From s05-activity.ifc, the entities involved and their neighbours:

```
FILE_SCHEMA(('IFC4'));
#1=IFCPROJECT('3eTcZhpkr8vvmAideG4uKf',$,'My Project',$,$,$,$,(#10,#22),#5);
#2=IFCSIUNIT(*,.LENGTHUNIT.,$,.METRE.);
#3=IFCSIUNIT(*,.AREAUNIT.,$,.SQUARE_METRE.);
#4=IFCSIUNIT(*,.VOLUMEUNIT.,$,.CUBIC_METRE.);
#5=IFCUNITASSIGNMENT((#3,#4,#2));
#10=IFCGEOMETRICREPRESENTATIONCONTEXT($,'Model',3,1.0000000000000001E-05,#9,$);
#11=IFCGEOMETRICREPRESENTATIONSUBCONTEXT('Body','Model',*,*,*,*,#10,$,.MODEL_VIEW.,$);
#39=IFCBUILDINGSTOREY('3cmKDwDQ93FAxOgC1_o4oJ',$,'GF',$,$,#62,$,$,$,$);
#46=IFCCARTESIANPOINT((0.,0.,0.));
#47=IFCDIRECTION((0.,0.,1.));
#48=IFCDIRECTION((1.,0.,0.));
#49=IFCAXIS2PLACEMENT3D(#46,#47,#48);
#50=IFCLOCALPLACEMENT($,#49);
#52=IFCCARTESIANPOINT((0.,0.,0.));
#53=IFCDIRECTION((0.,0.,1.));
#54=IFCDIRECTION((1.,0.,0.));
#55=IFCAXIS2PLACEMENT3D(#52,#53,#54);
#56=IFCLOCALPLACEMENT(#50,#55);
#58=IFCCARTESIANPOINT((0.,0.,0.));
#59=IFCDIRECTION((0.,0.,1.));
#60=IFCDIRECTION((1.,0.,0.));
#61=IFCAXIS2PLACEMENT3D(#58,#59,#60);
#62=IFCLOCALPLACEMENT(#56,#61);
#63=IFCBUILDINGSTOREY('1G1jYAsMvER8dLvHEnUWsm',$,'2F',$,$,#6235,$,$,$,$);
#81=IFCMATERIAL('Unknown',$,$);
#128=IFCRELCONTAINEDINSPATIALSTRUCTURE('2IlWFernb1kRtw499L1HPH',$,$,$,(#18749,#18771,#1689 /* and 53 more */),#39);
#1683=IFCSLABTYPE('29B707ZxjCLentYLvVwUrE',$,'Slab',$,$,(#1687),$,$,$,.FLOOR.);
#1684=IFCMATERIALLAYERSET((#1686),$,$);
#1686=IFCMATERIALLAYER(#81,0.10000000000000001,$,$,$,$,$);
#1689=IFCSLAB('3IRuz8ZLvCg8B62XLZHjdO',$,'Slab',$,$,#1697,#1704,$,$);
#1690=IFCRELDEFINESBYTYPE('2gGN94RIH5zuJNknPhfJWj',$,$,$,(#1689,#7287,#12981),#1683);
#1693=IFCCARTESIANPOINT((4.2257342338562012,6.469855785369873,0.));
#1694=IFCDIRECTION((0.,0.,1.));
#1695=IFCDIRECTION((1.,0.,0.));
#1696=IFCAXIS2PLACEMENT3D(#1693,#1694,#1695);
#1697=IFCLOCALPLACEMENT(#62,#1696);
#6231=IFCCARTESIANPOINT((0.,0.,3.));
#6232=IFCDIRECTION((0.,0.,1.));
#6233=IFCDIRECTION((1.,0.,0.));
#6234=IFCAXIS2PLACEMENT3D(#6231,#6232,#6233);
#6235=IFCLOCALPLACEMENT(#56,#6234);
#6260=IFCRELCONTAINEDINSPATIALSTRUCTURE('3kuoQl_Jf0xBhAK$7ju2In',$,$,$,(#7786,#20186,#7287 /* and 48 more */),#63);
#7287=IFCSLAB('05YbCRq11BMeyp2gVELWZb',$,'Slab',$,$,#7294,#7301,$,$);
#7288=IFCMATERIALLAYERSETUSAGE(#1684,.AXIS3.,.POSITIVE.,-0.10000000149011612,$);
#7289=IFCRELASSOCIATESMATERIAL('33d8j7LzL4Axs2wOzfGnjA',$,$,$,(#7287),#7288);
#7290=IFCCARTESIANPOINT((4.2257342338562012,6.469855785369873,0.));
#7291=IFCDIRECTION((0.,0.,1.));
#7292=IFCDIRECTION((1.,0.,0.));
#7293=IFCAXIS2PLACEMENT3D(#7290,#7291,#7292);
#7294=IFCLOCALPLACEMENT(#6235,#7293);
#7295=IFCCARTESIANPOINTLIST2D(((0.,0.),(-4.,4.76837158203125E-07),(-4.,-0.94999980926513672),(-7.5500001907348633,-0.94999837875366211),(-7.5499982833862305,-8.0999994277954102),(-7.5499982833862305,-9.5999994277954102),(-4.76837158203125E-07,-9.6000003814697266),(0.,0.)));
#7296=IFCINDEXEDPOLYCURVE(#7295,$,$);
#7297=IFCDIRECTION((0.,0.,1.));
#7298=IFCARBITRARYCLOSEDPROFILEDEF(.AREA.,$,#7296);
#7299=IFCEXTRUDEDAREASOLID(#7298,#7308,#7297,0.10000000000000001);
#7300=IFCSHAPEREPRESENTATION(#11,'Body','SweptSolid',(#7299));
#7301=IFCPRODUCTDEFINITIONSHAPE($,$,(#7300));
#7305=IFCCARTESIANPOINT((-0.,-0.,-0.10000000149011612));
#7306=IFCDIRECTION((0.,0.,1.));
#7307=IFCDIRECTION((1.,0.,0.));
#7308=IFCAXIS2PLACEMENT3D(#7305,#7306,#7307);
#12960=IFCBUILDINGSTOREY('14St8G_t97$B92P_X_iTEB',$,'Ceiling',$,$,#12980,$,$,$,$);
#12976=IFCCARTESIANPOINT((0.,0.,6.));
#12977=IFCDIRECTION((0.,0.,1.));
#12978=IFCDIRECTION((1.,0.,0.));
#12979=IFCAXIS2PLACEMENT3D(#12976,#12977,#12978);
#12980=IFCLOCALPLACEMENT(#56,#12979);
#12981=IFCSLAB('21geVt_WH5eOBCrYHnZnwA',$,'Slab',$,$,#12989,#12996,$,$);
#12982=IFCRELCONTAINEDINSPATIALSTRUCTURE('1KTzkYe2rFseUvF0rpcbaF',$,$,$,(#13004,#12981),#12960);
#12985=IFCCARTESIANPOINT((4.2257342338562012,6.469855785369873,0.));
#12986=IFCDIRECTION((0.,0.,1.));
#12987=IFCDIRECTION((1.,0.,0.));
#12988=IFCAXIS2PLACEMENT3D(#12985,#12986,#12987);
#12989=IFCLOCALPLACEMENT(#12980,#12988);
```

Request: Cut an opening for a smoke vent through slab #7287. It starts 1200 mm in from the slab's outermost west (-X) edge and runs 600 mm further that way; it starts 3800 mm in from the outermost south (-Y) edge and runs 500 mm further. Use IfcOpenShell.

```python
import numpy as np
import ifcopenshell
import ifcopenshell.api.feature
import ifcopenshell.api.geometry
import ifcopenshell.api.root
import ifcopenshell.geom
import ifcopenshell.util.placement
import ifcopenshell.util.representation
import ifcopenshell.util.shape
import ifcopenshell.util.unit

model = ifcopenshell.open("s05-activity.ifc")
unit_scale = ifcopenshell.util.unit.calculate_unit_scale(model)
settings = ifcopenshell.geom.settings()


def volume(element):
    """Net volume in cubic metres, openings subtracted."""
    shape = ifcopenshell.geom.create_shape(settings, element)
    return ifcopenshell.util.shape.get_volume(shape.geometry)


slab = model.by_id(7287)
before = volume(slab)

# Extent in the slab's own axes, in metres. The edges named are its -X and -Y sides.
slab_shape = ifcopenshell.geom.create_shape(settings, slab)
vertices = ifcopenshell.util.shape.get_vertices(slab_shape.geometry)
x_min, y_min, bottom = vertices.min(axis=0)
top = vertices[:, 2].max()

opening = ifcopenshell.api.root.create_entity(model, ifc_class="IfcOpeningElement", name="Smoke vent opening", predefined_type="OPENING")
context = ifcopenshell.util.representation.get_context(model, "Model", "Body", "MODEL_VIEW")
width, depth = 0.6, 0.5
outline = [(0.0, 0.0), (width, 0.0), (width, depth), (0.0, depth), (0.0, 0.0)]
# Overshoot both faces by 50 mm so the cut is clean.
shape = ifcopenshell.api.geometry.add_slab_representation(
    model, context=context, depth=top - bottom + 0.1, polyline=outline
)
ifcopenshell.api.geometry.assign_representation(model, product=opening, representation=shape)

matrix = ifcopenshell.util.placement.get_local_placement(slab.ObjectPlacement)
matrix[:, 3] = matrix @ np.append(np.array([x_min + 1.2, y_min + 3.8, bottom - 0.05]) / unit_scale, 1.0)
ifcopenshell.api.geometry.edit_object_placement(model, product=opening, matrix=matrix, is_si=False)
ifcopenshell.api.feature.add_feature(model, feature=opening, element=slab)

after = volume(slab)

print(f"slab volume {before:.3f} -> {after:.3f} m3")

model.write("s05-activity_updated.ifc")
```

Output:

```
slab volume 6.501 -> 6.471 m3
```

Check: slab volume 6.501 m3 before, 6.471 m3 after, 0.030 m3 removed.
